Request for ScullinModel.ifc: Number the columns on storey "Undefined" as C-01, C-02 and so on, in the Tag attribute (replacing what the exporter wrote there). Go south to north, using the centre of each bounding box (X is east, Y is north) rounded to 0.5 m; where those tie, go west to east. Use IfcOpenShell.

First a look at what the model holds.

```python
import ifcopenshell
import ifcopenshell.util.element
import ifcopenshell.util.placement

model = ifcopenshell.open("ScullinModel.ifc")
print(model.schema)
storey = next(s for s in model.by_type("IfcBuildingStorey") if s.Name == "Undefined")
columns = [e for e in ifcopenshell.util.element.get_decomposition(storey) if e.is_a("IfcColumn")]
for e in sorted(columns, key=lambda e: e.id()):
    origin = ifcopenshell.util.placement.get_local_placement(e.ObjectPlacement)[:3, 3]
    print(e.id(), e.Tag, e.Name, origin.round(2) + 0.0, sep=" | ")
```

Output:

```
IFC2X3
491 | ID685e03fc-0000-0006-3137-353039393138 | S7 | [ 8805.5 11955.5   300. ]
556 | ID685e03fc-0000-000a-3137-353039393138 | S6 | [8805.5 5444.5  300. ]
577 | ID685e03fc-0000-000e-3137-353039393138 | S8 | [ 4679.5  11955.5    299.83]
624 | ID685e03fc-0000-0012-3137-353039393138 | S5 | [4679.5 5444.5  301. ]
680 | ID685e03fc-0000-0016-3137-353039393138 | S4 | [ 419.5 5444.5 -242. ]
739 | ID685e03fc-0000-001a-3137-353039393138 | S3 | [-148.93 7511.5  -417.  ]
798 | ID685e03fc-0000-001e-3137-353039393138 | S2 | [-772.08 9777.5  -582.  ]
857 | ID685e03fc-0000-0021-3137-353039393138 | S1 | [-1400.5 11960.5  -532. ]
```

```python
import ifcopenshell
import ifcopenshell.geom
import ifcopenshell.util.element
import ifcopenshell.util.shape

model = ifcopenshell.open("ScullinModel.ifc")
settings = ifcopenshell.geom.settings()
settings.set("use-world-coords", True)


def centre(element):
    shape = ifcopenshell.geom.create_shape(settings, element)
    return ifcopenshell.util.shape.get_bbox_centroid(shape.geometry)


storey = next(s for s in model.by_type("IfcBuildingStorey") if s.Name == "Undefined")
columns = [e for e in ifcopenshell.util.element.get_decomposition(storey) if e.is_a("IfcColumn")]

# Insertion points can sit at a corner or the storey origin, so sort by the geometry (in metres).
centres = {e: centre(e) for e in columns}
columns.sort(key=lambda e: (round(centres[e][1] / 0.5), centres[e][0]))

for i, e in enumerate(columns, start=1):
    number = f"C-{i:02d}"
    e.Tag = number
    print(e.id(), number)

model.write("ScullinModel_v2.ifc")
```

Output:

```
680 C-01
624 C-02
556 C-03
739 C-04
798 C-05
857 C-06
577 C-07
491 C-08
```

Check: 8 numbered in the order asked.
